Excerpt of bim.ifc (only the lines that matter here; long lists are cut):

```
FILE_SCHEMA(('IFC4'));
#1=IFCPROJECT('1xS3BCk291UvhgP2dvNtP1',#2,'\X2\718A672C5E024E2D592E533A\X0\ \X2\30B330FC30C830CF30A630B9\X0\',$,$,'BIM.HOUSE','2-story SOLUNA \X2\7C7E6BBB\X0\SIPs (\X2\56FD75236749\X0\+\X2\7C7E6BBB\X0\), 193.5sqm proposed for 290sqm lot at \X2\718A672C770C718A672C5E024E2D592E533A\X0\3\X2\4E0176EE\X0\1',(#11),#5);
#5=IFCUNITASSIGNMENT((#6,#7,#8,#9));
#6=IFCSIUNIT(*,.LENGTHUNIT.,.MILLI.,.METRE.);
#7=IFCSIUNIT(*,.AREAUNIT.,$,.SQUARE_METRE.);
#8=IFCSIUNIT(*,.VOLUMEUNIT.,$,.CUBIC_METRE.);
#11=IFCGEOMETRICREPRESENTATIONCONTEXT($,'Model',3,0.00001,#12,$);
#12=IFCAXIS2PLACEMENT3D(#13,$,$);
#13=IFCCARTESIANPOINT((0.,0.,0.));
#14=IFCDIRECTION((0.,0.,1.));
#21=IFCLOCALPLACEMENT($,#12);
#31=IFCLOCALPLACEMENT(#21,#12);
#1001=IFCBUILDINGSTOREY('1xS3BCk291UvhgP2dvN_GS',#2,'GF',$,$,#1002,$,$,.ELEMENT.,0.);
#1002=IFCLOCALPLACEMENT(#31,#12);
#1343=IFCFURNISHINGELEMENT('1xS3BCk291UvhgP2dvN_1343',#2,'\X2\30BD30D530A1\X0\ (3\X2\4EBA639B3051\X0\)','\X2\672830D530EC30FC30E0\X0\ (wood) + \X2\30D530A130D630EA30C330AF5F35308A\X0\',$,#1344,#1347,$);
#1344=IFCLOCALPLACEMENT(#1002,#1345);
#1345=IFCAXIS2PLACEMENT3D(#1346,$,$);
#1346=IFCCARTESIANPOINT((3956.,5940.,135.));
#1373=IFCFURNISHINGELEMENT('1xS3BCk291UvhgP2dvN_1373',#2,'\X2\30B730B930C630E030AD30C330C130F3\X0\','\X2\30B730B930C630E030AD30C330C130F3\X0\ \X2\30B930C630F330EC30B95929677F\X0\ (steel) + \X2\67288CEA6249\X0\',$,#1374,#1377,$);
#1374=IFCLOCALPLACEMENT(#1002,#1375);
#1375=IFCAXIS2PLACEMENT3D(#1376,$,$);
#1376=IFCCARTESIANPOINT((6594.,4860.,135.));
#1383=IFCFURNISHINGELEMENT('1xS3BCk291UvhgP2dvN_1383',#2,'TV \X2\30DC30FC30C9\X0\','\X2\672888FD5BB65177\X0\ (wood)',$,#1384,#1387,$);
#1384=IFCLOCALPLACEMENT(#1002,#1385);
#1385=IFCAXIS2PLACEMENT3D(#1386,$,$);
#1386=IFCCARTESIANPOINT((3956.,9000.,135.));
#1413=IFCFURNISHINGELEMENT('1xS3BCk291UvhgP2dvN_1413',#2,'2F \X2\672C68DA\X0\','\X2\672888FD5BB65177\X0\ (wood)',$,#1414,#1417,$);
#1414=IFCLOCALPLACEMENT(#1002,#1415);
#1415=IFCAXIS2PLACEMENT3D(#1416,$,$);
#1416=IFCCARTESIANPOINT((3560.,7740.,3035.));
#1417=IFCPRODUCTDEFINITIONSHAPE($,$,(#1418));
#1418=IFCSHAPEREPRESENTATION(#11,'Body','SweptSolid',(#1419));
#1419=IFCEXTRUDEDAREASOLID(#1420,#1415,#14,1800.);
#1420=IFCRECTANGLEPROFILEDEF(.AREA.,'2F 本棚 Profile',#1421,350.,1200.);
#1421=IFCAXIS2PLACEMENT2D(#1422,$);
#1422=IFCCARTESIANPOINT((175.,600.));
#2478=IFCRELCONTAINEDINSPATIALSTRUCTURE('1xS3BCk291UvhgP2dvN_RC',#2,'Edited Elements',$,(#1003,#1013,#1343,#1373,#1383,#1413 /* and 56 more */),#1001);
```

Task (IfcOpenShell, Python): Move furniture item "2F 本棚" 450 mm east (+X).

```python
import ifcopenshell
import ifcopenshell.api.geometry
import ifcopenshell.util.placement

model = ifcopenshell.open("bim.ifc")

item = model.by_guid("1xS3BCk291UvhgP2dvN_1413")
matrix = ifcopenshell.util.placement.get_local_placement(item.ObjectPlacement)
matrix[0, 3] += 450.0
ifcopenshell.api.geometry.edit_object_placement(model, product=item, matrix=matrix, is_si=False)

print(ifcopenshell.util.placement.get_local_placement(item.ObjectPlacement).round(3) + 0.0)

model.write("bim-out.ifc")
```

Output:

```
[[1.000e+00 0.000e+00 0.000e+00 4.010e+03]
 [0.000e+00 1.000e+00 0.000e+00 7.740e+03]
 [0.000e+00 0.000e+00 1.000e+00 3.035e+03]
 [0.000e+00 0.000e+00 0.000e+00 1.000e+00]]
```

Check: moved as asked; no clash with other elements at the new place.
